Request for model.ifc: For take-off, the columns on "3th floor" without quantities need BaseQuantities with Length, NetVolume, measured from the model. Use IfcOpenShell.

First a look at what the model holds.

```python
import ifcopenshell
import ifcopenshell.util.element
import ifcopenshell.util.unit

model = ifcopenshell.open("model.ifc")
print(model.schema)
for unit_type in ("LENGTHUNIT", "AREAUNIT", "VOLUMEUNIT"):
    print(unit_type, ifcopenshell.util.unit.calculate_unit_scale(model, unit_type))
storey = next(s for s in model.by_type("IfcBuildingStorey") if s.Name == "3th floor")
columns = [e for e in ifcopenshell.util.element.get_decomposition(storey) if e.is_a("IfcColumn")]
for e in sorted(columns, key=lambda e: e.id()):
    print(e.id(), e.is_a(), e.Name, list(ifcopenshell.util.element.get_psets(e, qtos_only=True)), sep=" | ")
```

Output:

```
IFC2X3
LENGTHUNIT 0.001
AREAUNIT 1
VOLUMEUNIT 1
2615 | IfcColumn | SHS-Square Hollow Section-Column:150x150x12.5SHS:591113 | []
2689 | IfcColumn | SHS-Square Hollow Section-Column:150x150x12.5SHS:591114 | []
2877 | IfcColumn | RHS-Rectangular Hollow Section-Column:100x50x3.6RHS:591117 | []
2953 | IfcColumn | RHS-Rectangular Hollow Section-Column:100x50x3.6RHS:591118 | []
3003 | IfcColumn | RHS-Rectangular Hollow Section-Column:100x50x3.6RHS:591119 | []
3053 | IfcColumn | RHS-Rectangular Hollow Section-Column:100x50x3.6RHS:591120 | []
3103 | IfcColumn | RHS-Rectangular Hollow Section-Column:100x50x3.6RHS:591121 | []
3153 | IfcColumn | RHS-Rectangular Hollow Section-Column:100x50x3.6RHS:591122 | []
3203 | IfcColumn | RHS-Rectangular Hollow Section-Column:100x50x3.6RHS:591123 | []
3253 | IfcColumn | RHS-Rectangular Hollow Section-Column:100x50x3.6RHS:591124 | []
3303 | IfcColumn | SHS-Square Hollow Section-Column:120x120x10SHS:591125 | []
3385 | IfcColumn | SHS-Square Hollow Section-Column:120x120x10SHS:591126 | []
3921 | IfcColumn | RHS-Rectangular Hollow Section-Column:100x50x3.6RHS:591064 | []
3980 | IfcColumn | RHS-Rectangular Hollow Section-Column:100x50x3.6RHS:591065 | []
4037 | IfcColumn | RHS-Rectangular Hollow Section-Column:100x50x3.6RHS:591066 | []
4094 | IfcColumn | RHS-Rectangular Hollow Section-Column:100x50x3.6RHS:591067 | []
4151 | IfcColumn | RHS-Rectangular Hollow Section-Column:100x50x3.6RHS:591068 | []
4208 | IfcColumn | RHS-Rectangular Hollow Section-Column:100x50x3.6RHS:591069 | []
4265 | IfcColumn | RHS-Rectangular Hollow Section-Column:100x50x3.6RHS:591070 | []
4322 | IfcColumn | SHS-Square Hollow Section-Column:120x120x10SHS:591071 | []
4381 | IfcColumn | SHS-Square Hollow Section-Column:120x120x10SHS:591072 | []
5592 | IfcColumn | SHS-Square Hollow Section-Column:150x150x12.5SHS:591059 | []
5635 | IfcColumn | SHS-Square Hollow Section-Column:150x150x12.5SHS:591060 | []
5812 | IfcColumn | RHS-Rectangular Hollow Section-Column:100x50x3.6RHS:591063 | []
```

```python
import ifcopenshell
import ifcopenshell.api.pset
import ifcopenshell.geom
import ifcopenshell.util.element
import ifcopenshell.util.shape
import ifcopenshell.util.unit

model = ifcopenshell.open("model.ifc")
unit_scale = ifcopenshell.util.unit.calculate_unit_scale(model)
volume_scale = ifcopenshell.util.unit.calculate_unit_scale(model, "VOLUMEUNIT")
settings = ifcopenshell.geom.settings()

storey = next(s for s in model.by_type("IfcBuildingStorey") if s.Name == "3th floor")
columns = [e for e in ifcopenshell.util.element.get_decomposition(storey) if e.is_a("IfcColumn")]

for e in sorted(columns, key=lambda e: e.id()):
    if ifcopenshell.util.element.get_psets(e, qtos_only=True, should_inherit=False):
        continue
    # Geometry comes back in metres, in the element's own axes.
    shape = ifcopenshell.geom.create_shape(settings, e)
    values = {
        "Length": ifcopenshell.util.shape.get_z(shape.geometry) / unit_scale,
        "NetVolume": ifcopenshell.util.shape.get_volume(shape.geometry) / volume_scale,
    }
    qto = ifcopenshell.api.pset.add_qto(model, product=e, name="BaseQuantities")
    ifcopenshell.api.pset.edit_qto(model, qto=qto, properties=values)
    print(e.id(), {k: round(v, 3) for k, v in values.items()})

model.write("model_updated.ifc")
```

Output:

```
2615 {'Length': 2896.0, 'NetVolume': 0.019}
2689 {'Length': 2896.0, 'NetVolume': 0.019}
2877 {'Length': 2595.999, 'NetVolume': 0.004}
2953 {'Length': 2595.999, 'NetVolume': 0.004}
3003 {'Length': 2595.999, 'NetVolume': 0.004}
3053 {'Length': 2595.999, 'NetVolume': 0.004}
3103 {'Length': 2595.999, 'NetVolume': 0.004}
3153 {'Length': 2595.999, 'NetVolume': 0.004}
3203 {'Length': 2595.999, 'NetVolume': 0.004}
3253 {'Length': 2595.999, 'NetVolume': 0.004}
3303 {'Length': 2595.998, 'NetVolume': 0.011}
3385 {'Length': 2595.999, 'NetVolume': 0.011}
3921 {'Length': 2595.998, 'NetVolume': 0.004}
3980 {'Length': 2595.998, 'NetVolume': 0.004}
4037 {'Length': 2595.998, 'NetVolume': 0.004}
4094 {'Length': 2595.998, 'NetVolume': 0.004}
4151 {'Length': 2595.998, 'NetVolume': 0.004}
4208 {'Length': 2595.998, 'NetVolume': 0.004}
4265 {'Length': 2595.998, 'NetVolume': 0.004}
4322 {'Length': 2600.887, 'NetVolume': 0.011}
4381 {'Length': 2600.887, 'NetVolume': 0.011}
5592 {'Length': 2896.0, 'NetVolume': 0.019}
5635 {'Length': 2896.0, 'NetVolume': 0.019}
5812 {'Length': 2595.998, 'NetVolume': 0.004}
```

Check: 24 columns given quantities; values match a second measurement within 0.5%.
